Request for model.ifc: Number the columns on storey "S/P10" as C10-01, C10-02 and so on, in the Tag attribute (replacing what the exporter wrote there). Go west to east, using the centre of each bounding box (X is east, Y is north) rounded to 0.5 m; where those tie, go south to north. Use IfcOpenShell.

First a look at what the model holds.

```python
import ifcopenshell
import ifcopenshell.util.element
import ifcopenshell.util.placement

model = ifcopenshell.open("model.ifc")
print(model.schema)
storey = next(s for s in model.by_type("IfcBuildingStorey") if s.Name == "S/P10")
columns = [e for e in ifcopenshell.util.element.get_decomposition(storey) if e.is_a("IfcColumn")]
for e in sorted(columns, key=lambda e: e.id()):
    origin = ifcopenshell.util.placement.get_local_placement(e.ObjectPlacement)[:3, 3]
    print(e.id(), e.Tag, e.Name, origin.round(2) + 0.0, sep=" | ")
```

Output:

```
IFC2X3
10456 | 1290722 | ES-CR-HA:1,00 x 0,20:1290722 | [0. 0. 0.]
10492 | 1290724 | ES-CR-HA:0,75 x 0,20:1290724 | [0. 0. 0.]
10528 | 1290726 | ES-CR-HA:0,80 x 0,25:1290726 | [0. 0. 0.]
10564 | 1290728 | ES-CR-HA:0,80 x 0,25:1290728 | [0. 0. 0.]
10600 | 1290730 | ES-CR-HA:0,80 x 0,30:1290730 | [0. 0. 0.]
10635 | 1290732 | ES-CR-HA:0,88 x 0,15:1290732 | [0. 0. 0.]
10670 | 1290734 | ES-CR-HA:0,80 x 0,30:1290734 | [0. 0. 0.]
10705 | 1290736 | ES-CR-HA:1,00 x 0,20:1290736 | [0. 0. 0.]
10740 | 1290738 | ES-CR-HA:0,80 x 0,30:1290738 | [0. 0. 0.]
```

```python
import ifcopenshell
import ifcopenshell.geom
import ifcopenshell.util.element
import ifcopenshell.util.shape

model = ifcopenshell.open("model.ifc")
settings = ifcopenshell.geom.settings()
settings.set("use-world-coords", True)


def centre(element):
    shape = ifcopenshell.geom.create_shape(settings, element)
    return ifcopenshell.util.shape.get_bbox_centroid(shape.geometry)


storey = next(s for s in model.by_type("IfcBuildingStorey") if s.Name == "S/P10")
columns = [e for e in ifcopenshell.util.element.get_decomposition(storey) if e.is_a("IfcColumn")]

# Insertion points can sit at a corner or the storey origin, so sort by the geometry (in metres).
centres = {e: centre(e) for e in columns}
columns.sort(key=lambda e: (round(centres[e][0] / 0.5), centres[e][1]))

for i, e in enumerate(columns, start=1):
    number = f"C10-{i:02d}"
    e.Tag = number
    print(e.id(), number)

model.write("model_v2.ifc")
```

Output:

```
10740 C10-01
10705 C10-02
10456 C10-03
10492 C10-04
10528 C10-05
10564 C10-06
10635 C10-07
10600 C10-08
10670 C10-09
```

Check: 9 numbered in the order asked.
